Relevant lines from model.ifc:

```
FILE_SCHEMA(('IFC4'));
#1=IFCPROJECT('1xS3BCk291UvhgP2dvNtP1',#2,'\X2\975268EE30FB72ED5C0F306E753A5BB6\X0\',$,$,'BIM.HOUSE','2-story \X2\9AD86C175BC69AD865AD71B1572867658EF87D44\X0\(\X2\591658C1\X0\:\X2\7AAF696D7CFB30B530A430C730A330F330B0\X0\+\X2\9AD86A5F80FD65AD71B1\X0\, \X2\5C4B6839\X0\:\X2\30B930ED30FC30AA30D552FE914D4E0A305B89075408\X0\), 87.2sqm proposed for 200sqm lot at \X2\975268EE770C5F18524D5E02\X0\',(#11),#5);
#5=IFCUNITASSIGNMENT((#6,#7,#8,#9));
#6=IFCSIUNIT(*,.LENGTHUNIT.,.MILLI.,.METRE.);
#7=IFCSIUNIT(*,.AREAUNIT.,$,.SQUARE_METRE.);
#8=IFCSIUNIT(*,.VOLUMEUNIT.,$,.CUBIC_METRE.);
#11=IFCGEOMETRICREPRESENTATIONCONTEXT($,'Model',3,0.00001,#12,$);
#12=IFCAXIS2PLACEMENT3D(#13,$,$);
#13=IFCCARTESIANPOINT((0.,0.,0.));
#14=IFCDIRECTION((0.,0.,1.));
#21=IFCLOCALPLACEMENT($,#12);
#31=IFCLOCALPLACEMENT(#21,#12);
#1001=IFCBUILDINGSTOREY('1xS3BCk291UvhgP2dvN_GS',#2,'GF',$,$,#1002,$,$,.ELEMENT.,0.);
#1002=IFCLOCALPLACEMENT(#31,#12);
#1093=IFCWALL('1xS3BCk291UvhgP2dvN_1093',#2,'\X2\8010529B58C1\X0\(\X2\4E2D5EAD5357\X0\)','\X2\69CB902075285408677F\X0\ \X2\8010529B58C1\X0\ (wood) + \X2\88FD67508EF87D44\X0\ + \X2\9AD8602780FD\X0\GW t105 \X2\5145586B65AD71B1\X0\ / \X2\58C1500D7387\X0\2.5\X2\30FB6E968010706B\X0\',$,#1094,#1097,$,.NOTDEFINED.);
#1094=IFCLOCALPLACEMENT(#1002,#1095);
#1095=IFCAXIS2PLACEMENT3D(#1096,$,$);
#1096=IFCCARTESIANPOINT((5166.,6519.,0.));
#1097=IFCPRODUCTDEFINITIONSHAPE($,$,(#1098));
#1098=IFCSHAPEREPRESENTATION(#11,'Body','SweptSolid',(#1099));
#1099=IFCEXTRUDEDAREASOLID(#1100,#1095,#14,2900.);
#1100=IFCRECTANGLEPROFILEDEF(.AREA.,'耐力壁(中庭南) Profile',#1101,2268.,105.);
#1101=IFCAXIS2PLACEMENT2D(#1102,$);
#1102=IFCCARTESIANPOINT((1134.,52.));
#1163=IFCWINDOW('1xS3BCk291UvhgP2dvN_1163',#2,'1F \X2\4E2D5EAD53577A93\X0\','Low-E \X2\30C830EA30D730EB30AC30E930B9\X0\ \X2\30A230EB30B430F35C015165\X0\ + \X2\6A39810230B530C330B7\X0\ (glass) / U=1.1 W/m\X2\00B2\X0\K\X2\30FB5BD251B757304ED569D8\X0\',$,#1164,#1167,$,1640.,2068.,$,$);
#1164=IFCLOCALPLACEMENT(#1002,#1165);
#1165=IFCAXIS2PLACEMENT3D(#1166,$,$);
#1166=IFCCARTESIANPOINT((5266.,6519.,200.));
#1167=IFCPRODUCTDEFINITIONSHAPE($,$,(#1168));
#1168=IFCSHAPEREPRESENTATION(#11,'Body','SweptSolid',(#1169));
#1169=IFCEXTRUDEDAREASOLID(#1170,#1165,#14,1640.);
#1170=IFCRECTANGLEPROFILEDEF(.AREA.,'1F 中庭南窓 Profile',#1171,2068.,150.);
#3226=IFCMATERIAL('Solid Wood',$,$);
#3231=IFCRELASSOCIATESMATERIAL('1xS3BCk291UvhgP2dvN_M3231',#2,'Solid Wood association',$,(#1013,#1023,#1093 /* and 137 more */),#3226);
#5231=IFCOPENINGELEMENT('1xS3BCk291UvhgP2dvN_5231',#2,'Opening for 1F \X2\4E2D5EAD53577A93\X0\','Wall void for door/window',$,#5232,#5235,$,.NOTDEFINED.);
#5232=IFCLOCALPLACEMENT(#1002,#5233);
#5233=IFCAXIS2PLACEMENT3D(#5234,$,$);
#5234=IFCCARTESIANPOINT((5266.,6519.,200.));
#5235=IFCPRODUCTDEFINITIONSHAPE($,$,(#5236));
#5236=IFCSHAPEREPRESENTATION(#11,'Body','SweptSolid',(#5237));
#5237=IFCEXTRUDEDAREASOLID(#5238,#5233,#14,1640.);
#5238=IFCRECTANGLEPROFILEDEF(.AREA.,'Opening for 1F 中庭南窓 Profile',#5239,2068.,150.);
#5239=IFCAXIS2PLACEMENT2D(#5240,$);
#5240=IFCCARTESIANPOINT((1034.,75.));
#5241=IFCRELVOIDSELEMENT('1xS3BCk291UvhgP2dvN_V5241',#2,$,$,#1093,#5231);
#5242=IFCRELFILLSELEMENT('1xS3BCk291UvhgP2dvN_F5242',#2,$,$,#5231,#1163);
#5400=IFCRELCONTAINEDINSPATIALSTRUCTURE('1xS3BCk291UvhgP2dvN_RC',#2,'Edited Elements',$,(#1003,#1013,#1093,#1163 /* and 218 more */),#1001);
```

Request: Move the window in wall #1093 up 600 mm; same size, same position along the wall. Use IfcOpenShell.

```python
import numpy as np
import ifcopenshell
import ifcopenshell.api.geometry
import ifcopenshell.util.placement
import ifcopenshell.util.unit

model = ifcopenshell.open("model.ifc")
unit_scale = ifcopenshell.util.unit.calculate_unit_scale(model)

window = model.by_id(1163)
opening = window.FillsVoids[0].RelatingOpeningElement
dz = 0.6 / unit_scale

shift = np.array([0.0, 0.0, dz])
# The window is not placed relative to its opening, so move both.
for product in (opening, window):
    matrix = ifcopenshell.util.placement.get_local_placement(product.ObjectPlacement)
    matrix[:3, 3] += shift
    ifcopenshell.api.geometry.edit_object_placement(model, product=product, matrix=matrix, is_si=False)

print(f"moved by {dz * unit_scale:+.3f} m")

model.write("model_edited.ifc")
```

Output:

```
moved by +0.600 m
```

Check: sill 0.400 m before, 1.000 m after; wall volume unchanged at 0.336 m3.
